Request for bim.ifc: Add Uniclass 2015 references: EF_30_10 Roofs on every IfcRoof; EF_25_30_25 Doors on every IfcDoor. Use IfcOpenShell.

First a look at what the model holds.

```python
import ifcopenshell

model = ifcopenshell.open("bim.ifc")
print(model.schema)
print("classifications:", [c.Name for c in model.by_type("IfcClassification")])
for ifc_class in ("IfcDoor", "IfcRoof", "IfcStair", "IfcWall", "IfcWindow"):
    print(ifc_class, len(model.by_type(ifc_class)))
```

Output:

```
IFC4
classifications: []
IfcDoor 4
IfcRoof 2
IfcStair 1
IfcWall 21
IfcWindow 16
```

```python
import ifcopenshell
import ifcopenshell.api.classification

model = ifcopenshell.open("bim.ifc")

system = ifcopenshell.api.classification.add_classification(model, classification="Uniclass 2015")

codes = {
    "IfcRoof": ("EF_30_10", "Roofs"),
    "IfcDoor": ("EF_25_30_25", "Doors"),
}
for ifc_class, (code, name) in codes.items():
    products = model.by_type(ifc_class)
    ifcopenshell.api.classification.add_reference(
        model, products=products, classification=system, identification=code, name=name
    )
    print(code, len(products))

model.write("bim_edited.ifc")
```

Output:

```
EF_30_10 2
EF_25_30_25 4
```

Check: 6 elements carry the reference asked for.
